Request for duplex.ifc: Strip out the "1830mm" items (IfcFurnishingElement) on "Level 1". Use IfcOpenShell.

First a look at what the model holds.

```python
import ifcopenshell
import ifcopenshell.util.element

model = ifcopenshell.open("duplex.ifc")
print(model.schema)
storey = next(s for s in model.by_type("IfcBuildingStorey") if s.Name == "Level 1")
furniture = [e for e in ifcopenshell.util.element.get_decomposition(storey) if e.is_a("IfcFurnishingElement")]
seen = {}
for e in furniture:
    element_type = ifcopenshell.util.element.get_type(e)
    name = element_type.Name if element_type not in (None, e) else None
    seen[name] = seen.get(name, 0) + 1
for name, count in sorted(seen.items(), key=str):
    print(count, "x", name)
```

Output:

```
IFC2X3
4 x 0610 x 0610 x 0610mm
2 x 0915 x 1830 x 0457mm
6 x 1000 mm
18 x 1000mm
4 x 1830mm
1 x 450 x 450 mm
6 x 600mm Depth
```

```python
import ifcopenshell
import ifcopenshell.api.root
import ifcopenshell.util.element

model = ifcopenshell.open("duplex.ifc")

storey = next(s for s in model.by_type("IfcBuildingStorey") if s.Name == "Level 1")
furniture = [e for e in ifcopenshell.util.element.get_decomposition(storey) if e.is_a("IfcFurnishingElement")]
targets = [e for e in furniture if (t := ifcopenshell.util.element.get_type(e)) not in (None, e) and t.Name == "1830mm"]

for e in targets:
    ifcopenshell.api.root.remove_product(model, product=e)
print(len(targets), "removed")

model.write("duplex_edited.ifc")
```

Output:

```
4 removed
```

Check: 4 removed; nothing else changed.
